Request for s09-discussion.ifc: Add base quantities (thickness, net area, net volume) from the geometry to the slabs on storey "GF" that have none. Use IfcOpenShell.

First a look at what the model holds.

```python
import ifcopenshell
import ifcopenshell.util.element
import ifcopenshell.util.unit

model = ifcopenshell.open("s09-discussion.ifc")
print(model.schema)
for unit_type in ("LENGTHUNIT", "AREAUNIT", "VOLUMEUNIT"):
    print(unit_type, ifcopenshell.util.unit.calculate_unit_scale(model, unit_type))
storey = next(s for s in model.by_type("IfcBuildingStorey") if s.Name == "GF")
slabs = [e for e in ifcopenshell.util.element.get_decomposition(storey) if e.is_a("IfcSlab")]
for e in sorted(slabs, key=lambda e: e.id()):
    print(e.id(), e.is_a(), e.Name, list(ifcopenshell.util.element.get_psets(e, qtos_only=True)), sep=" | ")
```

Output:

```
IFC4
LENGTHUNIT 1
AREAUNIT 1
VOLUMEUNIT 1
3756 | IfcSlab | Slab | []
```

```python
import ifcopenshell
import ifcopenshell.api.pset
import ifcopenshell.geom
import ifcopenshell.util.element
import ifcopenshell.util.shape
import ifcopenshell.util.unit

model = ifcopenshell.open("s09-discussion.ifc")
unit_scale = ifcopenshell.util.unit.calculate_unit_scale(model)
area_scale = ifcopenshell.util.unit.calculate_unit_scale(model, "AREAUNIT")
volume_scale = ifcopenshell.util.unit.calculate_unit_scale(model, "VOLUMEUNIT")
settings = ifcopenshell.geom.settings()

storey = next(s for s in model.by_type("IfcBuildingStorey") if s.Name == "GF")
slabs = [e for e in ifcopenshell.util.element.get_decomposition(storey) if e.is_a("IfcSlab")]

for e in sorted(slabs, key=lambda e: e.id()):
    if ifcopenshell.util.element.get_psets(e, qtos_only=True, should_inherit=False):
        continue
    # Geometry comes back in metres, in the element's own axes.
    shape = ifcopenshell.geom.create_shape(settings, e)
    values = {
        "Width": ifcopenshell.util.shape.get_z(shape.geometry) / unit_scale,
        "NetArea": ifcopenshell.util.shape.get_footprint_area(shape.geometry) / area_scale,
        "NetVolume": ifcopenshell.util.shape.get_volume(shape.geometry) / volume_scale,
    }
    qto = ifcopenshell.api.pset.add_qto(model, product=e, name="Qto_SlabBaseQuantities")
    ifcopenshell.api.pset.edit_qto(model, qto=qto, properties=values)
    print(e.id(), {k: round(v, 3) for k, v in values.items()})

model.write("s09-discussion_updated.ifc")
```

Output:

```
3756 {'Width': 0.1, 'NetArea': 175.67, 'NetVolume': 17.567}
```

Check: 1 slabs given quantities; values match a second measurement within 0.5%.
